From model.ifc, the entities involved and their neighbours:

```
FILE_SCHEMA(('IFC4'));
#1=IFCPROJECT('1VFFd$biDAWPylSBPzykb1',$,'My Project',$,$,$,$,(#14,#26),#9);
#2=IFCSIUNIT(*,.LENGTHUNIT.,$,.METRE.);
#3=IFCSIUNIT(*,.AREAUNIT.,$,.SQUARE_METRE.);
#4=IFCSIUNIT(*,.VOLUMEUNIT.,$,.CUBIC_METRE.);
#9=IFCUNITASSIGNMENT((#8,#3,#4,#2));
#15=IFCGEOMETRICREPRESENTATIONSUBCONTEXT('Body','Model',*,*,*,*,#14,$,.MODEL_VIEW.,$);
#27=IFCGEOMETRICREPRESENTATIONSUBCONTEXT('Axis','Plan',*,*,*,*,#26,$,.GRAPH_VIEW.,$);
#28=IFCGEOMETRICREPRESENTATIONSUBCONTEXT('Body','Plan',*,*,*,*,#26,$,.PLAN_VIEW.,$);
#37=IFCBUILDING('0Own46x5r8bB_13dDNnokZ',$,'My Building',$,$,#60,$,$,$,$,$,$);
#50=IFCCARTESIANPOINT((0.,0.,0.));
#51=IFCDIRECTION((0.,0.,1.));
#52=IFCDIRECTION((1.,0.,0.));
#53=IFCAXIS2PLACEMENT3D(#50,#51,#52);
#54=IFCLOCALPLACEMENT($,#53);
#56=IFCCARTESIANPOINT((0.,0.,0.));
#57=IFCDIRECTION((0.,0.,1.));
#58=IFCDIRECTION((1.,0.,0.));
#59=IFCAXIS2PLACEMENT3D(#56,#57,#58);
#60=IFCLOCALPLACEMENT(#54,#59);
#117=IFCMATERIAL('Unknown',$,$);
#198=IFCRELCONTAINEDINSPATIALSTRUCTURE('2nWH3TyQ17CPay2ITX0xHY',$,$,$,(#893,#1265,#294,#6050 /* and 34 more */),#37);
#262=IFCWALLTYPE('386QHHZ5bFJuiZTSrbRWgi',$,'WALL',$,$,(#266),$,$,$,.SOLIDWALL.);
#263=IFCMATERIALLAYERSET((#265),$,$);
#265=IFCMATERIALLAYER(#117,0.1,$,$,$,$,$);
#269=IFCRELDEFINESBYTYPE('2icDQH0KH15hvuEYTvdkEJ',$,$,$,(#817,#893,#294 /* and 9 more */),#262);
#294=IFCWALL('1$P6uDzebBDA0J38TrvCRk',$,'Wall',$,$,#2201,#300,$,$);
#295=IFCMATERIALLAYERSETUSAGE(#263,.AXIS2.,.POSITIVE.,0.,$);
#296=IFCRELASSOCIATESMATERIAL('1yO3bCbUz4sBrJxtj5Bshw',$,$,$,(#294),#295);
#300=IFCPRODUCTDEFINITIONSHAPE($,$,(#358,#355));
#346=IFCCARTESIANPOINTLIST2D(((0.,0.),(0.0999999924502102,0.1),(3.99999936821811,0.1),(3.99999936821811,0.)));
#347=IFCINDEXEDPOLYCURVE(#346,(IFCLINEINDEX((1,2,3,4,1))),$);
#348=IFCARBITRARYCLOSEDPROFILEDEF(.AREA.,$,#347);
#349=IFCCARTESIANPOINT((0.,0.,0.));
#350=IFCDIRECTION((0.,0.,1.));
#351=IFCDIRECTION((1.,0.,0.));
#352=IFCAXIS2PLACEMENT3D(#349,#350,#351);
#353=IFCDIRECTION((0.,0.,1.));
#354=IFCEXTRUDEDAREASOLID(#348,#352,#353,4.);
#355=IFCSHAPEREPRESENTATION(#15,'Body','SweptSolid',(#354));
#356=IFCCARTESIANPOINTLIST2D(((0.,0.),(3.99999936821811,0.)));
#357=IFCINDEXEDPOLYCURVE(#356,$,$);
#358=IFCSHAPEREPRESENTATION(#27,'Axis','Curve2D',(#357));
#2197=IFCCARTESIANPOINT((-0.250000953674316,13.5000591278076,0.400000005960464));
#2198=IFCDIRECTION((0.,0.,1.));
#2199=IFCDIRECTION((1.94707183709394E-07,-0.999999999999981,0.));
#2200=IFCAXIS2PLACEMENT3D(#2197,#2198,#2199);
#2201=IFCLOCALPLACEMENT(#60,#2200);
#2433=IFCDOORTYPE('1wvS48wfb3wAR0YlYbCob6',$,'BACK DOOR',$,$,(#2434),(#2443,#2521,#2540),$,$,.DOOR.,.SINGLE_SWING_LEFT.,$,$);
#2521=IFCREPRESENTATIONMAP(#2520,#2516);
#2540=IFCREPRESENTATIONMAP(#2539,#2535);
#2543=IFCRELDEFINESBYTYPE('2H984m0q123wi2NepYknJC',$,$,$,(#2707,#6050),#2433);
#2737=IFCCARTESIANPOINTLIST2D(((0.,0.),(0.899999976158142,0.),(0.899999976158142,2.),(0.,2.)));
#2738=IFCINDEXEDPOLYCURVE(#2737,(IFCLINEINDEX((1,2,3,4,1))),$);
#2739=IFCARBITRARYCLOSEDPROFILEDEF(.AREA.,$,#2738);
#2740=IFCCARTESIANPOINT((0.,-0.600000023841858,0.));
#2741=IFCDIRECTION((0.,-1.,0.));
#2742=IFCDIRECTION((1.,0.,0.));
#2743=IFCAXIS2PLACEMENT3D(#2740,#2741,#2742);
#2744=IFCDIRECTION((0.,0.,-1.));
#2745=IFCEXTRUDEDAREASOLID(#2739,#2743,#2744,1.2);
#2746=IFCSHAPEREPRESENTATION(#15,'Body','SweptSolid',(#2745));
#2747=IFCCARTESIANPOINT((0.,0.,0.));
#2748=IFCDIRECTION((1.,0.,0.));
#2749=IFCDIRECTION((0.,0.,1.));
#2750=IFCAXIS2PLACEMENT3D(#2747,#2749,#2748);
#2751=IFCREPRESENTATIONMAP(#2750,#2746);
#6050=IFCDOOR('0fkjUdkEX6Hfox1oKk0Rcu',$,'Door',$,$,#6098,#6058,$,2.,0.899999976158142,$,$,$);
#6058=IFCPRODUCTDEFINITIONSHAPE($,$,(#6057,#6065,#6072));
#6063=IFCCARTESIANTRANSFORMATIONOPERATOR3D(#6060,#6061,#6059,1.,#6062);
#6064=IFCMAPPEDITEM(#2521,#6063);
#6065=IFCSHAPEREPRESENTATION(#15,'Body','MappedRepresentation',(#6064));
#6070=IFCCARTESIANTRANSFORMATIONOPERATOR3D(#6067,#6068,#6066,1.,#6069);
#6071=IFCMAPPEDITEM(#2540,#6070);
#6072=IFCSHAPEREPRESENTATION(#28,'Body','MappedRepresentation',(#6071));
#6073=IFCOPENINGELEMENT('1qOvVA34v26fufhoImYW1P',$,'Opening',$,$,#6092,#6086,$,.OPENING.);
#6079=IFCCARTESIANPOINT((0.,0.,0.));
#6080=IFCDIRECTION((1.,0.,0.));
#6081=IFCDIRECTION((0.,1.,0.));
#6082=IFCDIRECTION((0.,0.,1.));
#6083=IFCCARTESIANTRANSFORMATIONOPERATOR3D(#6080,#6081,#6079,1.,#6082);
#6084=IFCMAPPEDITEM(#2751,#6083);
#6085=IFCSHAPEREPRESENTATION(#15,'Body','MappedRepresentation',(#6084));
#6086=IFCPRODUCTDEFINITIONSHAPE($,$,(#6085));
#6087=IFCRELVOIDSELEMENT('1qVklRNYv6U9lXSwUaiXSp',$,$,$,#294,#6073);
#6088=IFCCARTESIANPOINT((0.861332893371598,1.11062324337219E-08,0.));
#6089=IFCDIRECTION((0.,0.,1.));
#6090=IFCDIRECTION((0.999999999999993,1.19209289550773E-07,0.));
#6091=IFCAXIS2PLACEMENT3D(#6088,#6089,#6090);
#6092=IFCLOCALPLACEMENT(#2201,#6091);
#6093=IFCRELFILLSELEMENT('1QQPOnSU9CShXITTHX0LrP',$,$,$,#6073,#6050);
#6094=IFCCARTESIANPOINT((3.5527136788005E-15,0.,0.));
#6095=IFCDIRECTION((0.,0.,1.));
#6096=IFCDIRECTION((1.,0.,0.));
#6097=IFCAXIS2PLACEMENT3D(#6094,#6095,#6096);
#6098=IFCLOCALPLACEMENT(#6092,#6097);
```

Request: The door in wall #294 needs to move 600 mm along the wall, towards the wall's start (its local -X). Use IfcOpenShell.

```python
import ifcopenshell
import ifcopenshell.api.geometry
import ifcopenshell.util.placement

model = ifcopenshell.open("model.ifc")

door = model.by_id(6050)
opening = door.FillsVoids[0].RelatingOpeningElement
wall = opening.VoidsElements[0].RelatingBuildingElement

wall_matrix = ifcopenshell.util.placement.get_local_placement(wall.ObjectPlacement)
shift = wall_matrix[:3, 0] * -0.6
before = ifcopenshell.util.placement.get_local_placement(door.ObjectPlacement)[:3, 3].copy()

# The door is placed relative to its opening, so it follows when the opening moves.
matrix = ifcopenshell.util.placement.get_local_placement(opening.ObjectPlacement)
matrix[:3, 3] += shift
ifcopenshell.api.geometry.edit_object_placement(
    model, product=opening, matrix=matrix, is_si=False, should_transform_children=True
)

after = ifcopenshell.util.placement.get_local_placement(door.ObjectPlacement)[:3, 3]
print("door moved by", (after - before).round(3) + 0.0)

model.write("model_v2.ifc")
```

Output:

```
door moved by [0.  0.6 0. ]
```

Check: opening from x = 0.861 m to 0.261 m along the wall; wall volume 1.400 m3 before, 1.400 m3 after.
